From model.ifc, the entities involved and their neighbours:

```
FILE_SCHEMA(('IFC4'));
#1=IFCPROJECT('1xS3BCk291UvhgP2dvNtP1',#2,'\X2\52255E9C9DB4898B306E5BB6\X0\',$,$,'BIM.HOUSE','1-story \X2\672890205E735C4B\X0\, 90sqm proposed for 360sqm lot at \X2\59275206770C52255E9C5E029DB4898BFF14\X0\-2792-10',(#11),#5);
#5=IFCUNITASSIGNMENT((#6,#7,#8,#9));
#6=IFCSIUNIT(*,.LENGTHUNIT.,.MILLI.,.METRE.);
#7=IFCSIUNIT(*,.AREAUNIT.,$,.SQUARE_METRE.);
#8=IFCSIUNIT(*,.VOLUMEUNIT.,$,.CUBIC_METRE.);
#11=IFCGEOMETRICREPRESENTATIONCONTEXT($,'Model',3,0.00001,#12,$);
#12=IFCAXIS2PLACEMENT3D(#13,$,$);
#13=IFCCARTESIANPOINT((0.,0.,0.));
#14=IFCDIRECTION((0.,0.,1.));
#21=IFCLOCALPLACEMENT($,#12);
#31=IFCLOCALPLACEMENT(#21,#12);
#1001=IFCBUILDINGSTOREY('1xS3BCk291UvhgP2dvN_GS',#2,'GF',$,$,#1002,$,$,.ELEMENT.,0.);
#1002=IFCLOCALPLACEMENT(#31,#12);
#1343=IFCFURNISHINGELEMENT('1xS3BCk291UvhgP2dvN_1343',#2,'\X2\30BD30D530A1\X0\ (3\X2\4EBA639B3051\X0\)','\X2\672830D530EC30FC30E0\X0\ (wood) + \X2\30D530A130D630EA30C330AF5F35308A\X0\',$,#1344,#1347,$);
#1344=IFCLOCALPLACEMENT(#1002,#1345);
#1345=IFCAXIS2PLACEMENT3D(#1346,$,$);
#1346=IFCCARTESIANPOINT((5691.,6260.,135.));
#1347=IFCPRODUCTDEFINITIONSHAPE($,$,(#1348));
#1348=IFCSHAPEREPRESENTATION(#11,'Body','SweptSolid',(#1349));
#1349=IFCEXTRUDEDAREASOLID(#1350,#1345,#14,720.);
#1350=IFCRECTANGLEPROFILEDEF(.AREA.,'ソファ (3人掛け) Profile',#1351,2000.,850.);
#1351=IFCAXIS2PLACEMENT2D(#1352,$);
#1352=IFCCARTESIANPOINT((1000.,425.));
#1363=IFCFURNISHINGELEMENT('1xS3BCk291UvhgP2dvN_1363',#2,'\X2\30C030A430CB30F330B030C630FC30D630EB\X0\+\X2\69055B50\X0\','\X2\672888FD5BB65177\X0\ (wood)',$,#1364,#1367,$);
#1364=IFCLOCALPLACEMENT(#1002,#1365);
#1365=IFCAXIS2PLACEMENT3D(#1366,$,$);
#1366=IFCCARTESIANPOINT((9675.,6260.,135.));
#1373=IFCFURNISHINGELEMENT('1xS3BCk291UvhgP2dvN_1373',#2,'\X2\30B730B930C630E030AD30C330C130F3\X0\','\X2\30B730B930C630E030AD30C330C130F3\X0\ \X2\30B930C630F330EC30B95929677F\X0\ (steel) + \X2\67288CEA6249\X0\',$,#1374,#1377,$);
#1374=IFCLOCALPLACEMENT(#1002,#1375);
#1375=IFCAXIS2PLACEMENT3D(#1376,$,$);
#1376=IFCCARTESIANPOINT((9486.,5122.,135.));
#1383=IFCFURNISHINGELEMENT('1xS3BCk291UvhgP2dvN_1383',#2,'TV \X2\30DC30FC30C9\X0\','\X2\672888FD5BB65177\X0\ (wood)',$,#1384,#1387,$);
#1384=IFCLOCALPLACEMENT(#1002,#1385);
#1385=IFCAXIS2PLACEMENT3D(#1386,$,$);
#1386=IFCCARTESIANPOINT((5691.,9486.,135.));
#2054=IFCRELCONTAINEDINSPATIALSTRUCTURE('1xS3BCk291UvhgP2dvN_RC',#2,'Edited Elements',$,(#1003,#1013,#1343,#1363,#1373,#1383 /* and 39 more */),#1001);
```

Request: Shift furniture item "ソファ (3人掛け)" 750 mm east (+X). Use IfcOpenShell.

```python
import ifcopenshell
import ifcopenshell.api.geometry
import ifcopenshell.util.placement
import ifcopenshell.util.unit

model = ifcopenshell.open("model.ifc")
unit_scale = ifcopenshell.util.unit.calculate_unit_scale(model)

item = model.by_id(1343)
matrix = ifcopenshell.util.placement.get_local_placement(item.ObjectPlacement)
matrix[0, 3] += 0.75 / unit_scale
ifcopenshell.api.geometry.edit_object_placement(model, product=item, matrix=matrix, is_si=False)

print(ifcopenshell.util.placement.get_local_placement(item.ObjectPlacement).round(3) + 0.0)

model.write("model_updated.ifc")
```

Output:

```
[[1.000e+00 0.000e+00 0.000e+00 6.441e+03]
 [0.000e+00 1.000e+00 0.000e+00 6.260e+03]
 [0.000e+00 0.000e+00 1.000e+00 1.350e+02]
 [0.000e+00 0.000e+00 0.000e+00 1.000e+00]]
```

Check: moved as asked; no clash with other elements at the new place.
